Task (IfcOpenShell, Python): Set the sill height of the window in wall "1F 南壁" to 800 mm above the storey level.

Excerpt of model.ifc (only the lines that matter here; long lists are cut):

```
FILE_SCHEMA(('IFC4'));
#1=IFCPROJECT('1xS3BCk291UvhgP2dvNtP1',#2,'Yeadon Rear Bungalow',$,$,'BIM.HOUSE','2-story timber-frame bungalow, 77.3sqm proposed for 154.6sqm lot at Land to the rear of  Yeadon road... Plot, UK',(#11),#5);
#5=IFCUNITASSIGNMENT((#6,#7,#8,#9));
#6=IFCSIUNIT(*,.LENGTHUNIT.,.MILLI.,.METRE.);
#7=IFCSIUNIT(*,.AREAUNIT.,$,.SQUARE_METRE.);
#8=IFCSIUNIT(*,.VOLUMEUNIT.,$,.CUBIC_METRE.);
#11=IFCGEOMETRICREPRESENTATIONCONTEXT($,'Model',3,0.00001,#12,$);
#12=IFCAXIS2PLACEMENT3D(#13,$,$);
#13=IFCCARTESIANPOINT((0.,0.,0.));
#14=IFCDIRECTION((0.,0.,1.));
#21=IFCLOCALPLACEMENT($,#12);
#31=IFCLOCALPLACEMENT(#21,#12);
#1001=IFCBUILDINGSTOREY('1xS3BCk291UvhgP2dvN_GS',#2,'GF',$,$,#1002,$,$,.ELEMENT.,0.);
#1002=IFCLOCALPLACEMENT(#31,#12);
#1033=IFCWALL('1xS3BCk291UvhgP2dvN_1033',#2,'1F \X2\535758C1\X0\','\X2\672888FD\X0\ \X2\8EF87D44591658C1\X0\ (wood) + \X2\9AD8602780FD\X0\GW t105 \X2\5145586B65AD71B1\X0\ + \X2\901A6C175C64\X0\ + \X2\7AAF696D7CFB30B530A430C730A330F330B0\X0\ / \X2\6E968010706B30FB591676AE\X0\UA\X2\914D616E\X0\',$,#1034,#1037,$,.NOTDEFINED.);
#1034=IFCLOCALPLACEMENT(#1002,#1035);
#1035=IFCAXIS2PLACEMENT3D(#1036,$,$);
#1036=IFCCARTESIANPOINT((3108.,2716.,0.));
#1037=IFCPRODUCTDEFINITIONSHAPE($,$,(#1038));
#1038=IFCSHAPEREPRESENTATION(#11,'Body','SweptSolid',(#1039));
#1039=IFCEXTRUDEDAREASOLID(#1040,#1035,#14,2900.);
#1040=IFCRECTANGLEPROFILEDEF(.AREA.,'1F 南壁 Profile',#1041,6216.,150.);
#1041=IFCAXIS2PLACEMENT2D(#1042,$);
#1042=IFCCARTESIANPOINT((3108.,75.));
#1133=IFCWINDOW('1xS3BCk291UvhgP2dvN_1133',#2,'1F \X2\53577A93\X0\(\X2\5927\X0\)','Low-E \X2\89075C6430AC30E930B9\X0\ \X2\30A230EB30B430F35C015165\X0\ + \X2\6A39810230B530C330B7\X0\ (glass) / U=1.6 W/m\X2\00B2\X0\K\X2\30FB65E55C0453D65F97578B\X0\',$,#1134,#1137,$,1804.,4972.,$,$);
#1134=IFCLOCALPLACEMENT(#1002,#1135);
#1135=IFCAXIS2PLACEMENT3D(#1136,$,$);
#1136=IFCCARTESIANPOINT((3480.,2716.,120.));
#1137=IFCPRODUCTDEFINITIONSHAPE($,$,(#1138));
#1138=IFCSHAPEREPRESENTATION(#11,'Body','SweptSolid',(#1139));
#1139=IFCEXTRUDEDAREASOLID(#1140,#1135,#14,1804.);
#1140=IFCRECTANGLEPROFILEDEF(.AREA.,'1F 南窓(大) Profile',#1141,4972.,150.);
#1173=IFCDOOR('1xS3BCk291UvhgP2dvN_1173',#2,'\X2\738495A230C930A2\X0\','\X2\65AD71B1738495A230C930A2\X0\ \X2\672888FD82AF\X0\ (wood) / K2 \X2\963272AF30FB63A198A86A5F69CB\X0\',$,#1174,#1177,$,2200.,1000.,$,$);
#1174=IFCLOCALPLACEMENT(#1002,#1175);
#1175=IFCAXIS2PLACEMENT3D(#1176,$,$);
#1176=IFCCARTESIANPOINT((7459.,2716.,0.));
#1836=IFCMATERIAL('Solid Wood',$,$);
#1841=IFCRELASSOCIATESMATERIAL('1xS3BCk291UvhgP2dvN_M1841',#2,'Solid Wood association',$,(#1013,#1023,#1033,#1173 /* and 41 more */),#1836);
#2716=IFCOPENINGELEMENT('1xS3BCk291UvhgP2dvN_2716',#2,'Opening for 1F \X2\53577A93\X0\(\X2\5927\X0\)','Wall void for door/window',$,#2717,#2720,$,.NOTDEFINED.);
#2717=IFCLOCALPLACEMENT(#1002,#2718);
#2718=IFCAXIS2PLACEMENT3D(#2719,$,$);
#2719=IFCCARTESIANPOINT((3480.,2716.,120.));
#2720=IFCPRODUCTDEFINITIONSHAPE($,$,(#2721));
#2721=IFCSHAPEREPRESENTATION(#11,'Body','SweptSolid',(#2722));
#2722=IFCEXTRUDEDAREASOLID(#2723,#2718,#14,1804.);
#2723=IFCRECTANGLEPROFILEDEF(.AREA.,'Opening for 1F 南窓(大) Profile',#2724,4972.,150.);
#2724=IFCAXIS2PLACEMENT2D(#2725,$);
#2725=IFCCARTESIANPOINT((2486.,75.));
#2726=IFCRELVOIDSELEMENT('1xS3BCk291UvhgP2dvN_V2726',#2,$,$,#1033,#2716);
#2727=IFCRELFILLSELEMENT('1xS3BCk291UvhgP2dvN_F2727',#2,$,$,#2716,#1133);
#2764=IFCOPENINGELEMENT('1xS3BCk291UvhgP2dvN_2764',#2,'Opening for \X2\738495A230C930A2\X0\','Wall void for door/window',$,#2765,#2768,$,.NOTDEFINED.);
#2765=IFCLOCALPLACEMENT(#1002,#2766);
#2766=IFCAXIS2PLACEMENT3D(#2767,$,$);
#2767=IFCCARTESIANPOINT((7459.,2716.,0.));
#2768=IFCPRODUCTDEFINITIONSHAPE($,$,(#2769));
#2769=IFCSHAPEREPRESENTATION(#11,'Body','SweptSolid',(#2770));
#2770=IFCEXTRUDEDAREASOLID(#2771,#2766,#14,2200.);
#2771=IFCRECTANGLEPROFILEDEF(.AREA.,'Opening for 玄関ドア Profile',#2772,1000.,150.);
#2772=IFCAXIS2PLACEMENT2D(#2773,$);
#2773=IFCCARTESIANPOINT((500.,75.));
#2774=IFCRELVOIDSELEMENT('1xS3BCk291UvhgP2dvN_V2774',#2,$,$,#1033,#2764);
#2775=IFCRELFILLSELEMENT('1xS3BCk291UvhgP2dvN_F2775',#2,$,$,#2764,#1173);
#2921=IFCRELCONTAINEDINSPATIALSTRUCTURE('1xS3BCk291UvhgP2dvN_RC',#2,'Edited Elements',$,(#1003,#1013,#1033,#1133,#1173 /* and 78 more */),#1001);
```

```python
import numpy as np
import ifcopenshell
import ifcopenshell.api.geometry
import ifcopenshell.geom
import ifcopenshell.util.element
import ifcopenshell.util.placement
import ifcopenshell.util.shape
import ifcopenshell.util.unit

model = ifcopenshell.open("model.ifc")
unit_scale = ifcopenshell.util.unit.calculate_unit_scale(model)

window = model.by_guid("1xS3BCk291UvhgP2dvN_1133")
opening = window.FillsVoids[0].RelatingOpeningElement
storey = ifcopenshell.util.element.get_container(window, ifc_class="IfcBuildingStorey")
level = ifcopenshell.util.placement.get_local_placement(storey.ObjectPlacement)[2, 3]

# The opening's origin need not be at the sill, so measure its lowest point.
shape = ifcopenshell.geom.create_shape(ifcopenshell.geom.settings(), opening)
bottom = ifcopenshell.util.shape.get_shape_bottom_elevation(shape, shape.geometry) / unit_scale
dz = level + 0.8 / unit_scale - bottom

shift = np.array([0.0, 0.0, dz])
# The window is not placed relative to its opening, so move both.
for product in (opening, window):
    matrix = ifcopenshell.util.placement.get_local_placement(product.ObjectPlacement)
    matrix[:3, 3] += shift
    ifcopenshell.api.geometry.edit_object_placement(model, product=product, matrix=matrix, is_si=False)

print(f"moved by {dz * unit_scale:+.3f} m")

model.write("model-out.ifc")
```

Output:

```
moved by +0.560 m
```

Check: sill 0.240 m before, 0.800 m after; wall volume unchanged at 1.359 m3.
